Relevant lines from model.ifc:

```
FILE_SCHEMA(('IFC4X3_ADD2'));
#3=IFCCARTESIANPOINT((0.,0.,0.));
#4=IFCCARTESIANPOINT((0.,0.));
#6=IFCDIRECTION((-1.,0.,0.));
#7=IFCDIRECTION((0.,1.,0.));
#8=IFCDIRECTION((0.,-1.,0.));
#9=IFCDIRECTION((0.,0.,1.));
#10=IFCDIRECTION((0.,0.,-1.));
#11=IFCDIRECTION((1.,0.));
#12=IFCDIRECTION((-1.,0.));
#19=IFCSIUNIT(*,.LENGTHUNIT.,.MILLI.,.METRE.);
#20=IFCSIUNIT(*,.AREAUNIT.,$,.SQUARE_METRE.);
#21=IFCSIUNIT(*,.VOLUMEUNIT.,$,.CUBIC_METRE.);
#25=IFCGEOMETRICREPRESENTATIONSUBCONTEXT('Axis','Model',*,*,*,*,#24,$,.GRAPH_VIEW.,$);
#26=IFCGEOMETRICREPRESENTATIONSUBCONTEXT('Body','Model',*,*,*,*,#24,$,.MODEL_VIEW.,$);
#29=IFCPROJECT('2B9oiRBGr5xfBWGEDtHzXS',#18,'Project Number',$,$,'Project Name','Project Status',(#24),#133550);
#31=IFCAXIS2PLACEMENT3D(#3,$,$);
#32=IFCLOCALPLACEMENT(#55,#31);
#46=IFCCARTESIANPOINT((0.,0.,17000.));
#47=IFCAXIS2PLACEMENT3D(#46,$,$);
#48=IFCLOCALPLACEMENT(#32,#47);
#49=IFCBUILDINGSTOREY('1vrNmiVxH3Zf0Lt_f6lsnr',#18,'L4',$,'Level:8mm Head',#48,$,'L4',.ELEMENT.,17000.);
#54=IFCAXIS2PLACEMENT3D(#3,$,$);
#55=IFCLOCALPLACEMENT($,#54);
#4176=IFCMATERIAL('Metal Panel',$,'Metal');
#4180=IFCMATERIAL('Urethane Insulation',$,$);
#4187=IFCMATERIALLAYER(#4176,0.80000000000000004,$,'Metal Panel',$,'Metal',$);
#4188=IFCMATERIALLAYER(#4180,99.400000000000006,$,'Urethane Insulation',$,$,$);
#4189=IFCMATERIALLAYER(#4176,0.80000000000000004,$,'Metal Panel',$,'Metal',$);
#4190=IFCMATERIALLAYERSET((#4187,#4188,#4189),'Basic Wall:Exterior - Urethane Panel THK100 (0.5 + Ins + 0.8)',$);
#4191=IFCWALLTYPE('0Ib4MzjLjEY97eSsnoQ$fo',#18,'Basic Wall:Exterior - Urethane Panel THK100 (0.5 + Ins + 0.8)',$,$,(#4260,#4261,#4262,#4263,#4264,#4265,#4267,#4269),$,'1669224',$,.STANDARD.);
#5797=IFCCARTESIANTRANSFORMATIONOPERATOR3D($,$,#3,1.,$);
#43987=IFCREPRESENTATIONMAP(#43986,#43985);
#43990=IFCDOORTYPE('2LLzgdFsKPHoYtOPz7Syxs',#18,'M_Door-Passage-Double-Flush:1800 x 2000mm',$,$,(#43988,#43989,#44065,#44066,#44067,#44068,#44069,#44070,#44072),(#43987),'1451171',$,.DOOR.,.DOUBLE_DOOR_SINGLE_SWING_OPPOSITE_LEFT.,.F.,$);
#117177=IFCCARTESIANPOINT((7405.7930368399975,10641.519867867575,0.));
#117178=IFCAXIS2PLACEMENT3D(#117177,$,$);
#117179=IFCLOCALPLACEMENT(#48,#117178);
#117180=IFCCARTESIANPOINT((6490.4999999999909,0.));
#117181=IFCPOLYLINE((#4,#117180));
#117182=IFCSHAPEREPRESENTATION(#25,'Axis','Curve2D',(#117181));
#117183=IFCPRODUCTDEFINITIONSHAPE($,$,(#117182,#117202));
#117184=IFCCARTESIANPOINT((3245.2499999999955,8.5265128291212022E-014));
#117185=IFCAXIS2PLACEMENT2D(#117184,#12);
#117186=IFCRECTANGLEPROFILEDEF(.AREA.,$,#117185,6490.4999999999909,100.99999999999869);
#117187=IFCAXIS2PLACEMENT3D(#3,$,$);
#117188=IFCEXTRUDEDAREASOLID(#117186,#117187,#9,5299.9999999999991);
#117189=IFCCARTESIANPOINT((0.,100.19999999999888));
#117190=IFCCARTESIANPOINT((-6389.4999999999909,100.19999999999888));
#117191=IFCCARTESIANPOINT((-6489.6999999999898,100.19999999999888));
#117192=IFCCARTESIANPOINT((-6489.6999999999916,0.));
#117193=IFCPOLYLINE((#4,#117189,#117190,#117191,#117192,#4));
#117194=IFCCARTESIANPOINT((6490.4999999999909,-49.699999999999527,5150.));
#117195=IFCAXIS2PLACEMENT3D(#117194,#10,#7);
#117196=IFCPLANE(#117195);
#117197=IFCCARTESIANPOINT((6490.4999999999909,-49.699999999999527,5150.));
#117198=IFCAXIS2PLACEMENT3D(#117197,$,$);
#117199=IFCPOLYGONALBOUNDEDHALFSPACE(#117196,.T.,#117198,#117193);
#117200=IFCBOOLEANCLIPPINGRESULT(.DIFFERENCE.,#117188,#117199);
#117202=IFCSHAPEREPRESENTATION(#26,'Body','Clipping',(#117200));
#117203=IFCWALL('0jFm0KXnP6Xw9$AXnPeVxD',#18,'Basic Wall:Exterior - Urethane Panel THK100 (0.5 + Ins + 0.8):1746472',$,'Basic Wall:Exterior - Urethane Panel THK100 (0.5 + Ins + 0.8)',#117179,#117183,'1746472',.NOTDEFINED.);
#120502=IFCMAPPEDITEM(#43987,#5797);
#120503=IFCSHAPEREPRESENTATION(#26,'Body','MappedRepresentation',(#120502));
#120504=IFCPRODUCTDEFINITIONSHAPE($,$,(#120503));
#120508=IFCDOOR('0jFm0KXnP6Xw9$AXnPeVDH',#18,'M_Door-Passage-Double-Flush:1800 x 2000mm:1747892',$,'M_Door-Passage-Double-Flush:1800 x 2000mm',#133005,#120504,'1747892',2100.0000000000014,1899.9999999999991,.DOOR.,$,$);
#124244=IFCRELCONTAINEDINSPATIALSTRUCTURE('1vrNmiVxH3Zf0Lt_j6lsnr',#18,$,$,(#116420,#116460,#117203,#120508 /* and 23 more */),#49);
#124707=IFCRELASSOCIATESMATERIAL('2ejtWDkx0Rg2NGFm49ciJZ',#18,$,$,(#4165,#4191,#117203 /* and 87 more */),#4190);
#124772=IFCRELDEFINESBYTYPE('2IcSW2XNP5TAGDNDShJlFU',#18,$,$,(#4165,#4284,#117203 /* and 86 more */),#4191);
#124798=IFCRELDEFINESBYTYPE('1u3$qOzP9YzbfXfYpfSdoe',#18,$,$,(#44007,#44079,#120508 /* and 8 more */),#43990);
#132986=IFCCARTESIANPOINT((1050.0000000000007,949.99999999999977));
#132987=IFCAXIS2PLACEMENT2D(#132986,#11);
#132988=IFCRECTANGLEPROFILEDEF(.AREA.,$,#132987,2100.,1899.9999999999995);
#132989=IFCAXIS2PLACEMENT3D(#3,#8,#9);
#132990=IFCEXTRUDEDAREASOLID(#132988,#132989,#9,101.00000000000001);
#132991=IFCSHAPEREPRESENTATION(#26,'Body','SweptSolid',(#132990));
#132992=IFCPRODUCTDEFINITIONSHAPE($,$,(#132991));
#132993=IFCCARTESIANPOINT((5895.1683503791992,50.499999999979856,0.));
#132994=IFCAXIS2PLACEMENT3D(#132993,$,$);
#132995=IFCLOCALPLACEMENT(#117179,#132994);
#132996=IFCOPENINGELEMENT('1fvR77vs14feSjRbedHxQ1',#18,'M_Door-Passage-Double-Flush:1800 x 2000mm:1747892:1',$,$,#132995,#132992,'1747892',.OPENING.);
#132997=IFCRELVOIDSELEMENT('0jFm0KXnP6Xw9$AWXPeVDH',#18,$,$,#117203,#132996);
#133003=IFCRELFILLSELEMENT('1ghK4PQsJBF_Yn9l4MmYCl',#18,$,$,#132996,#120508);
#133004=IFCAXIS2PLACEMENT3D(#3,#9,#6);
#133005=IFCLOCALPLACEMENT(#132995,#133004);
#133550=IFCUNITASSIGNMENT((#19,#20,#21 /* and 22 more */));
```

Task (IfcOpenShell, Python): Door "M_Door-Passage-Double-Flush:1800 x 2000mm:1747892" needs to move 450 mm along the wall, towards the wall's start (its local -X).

```python
import ifcopenshell
import ifcopenshell.api.geometry
import ifcopenshell.util.placement

model = ifcopenshell.open("model.ifc")

door = model.by_guid("0jFm0KXnP6Xw9$AXnPeVDH")
opening = door.FillsVoids[0].RelatingOpeningElement
wall = opening.VoidsElements[0].RelatingBuildingElement

wall_matrix = ifcopenshell.util.placement.get_local_placement(wall.ObjectPlacement)
shift = wall_matrix[:3, 0] * -450.0
before = ifcopenshell.util.placement.get_local_placement(door.ObjectPlacement)[:3, 3].copy()

# The door is placed relative to its opening, so it follows when the opening moves.
matrix = ifcopenshell.util.placement.get_local_placement(opening.ObjectPlacement)
matrix[:3, 3] += shift
ifcopenshell.api.geometry.edit_object_placement(
    model, product=opening, matrix=matrix, is_si=False, should_transform_children=True
)

after = ifcopenshell.util.placement.get_local_placement(door.ObjectPlacement)[:3, 3]
print("door moved by", (after - before).round(3) + 0.0)

model.write("model_v2.ifc")
```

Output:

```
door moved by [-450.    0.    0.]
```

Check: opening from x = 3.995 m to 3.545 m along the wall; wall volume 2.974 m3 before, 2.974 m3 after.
